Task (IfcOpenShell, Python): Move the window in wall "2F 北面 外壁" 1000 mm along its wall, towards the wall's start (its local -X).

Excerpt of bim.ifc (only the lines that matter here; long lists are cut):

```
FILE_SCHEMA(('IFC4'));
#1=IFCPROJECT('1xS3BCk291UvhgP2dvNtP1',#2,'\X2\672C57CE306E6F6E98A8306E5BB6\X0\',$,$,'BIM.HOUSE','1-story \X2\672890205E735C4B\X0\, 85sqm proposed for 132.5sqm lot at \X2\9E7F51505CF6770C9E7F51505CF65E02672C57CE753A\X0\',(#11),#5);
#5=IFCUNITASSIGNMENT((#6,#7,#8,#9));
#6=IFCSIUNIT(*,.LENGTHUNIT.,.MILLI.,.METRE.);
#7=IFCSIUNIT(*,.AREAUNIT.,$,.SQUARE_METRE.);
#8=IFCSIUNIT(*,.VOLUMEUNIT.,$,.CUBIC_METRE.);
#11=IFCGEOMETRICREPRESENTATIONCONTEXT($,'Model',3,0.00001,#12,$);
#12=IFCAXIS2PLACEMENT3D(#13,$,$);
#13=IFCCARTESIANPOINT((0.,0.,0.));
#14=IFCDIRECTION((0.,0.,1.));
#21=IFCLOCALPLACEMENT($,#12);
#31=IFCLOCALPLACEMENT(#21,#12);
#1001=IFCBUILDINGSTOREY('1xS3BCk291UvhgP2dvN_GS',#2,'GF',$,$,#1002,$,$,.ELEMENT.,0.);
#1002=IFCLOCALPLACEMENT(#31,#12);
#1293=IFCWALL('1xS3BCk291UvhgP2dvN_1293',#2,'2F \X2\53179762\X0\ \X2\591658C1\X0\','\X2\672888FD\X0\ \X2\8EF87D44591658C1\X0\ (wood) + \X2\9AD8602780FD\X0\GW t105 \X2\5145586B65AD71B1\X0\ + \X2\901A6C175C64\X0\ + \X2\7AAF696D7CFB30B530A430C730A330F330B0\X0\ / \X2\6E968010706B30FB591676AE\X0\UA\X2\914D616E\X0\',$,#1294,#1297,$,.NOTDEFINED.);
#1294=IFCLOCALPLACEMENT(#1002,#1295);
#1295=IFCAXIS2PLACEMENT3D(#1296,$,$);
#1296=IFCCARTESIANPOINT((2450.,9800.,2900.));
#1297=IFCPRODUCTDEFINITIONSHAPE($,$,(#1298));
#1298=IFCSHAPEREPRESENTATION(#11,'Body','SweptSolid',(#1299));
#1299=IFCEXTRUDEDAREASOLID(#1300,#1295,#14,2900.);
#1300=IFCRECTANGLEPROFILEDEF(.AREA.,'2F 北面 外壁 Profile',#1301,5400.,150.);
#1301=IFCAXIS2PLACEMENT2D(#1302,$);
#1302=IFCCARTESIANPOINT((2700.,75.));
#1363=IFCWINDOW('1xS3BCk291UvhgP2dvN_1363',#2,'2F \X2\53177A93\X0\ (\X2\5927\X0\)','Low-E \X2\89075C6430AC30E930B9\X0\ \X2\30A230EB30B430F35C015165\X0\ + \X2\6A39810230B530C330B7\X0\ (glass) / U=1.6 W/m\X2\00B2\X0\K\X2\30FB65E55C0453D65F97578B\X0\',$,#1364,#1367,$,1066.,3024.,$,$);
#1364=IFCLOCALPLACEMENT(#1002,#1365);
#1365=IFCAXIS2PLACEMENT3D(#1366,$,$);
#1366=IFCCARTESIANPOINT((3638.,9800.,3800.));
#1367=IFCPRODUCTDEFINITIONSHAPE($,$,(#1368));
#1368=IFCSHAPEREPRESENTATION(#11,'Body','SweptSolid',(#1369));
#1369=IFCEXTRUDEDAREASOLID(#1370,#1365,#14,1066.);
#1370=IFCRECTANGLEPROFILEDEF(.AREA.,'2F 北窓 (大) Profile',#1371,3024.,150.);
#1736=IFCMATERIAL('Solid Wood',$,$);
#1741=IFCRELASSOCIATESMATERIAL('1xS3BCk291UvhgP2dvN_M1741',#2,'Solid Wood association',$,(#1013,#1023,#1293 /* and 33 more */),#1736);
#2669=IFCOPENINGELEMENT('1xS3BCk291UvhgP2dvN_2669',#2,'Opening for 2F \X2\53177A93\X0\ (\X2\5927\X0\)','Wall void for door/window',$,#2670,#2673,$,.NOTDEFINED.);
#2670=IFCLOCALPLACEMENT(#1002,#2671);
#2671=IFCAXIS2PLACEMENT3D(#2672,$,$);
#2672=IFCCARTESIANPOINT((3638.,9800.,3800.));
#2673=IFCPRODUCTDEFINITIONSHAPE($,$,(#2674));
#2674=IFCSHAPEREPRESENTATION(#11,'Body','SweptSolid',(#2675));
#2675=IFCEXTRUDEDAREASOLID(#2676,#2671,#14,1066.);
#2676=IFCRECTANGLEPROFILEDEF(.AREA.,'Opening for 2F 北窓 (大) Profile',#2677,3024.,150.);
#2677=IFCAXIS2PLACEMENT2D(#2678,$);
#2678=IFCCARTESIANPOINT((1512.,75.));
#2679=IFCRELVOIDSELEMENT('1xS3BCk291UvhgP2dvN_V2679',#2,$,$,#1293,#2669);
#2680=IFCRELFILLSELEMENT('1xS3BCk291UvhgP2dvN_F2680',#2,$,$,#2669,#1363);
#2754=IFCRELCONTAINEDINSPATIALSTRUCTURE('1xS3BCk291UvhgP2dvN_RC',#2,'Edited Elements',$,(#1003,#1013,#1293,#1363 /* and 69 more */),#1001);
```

```python
import ifcopenshell
import ifcopenshell.api.geometry
import ifcopenshell.util.placement
import ifcopenshell.util.unit

model = ifcopenshell.open("bim.ifc")
unit_scale = ifcopenshell.util.unit.calculate_unit_scale(model)

window = model.by_id(1363)
opening = window.FillsVoids[0].RelatingOpeningElement
wall = opening.VoidsElements[0].RelatingBuildingElement

wall_matrix = ifcopenshell.util.placement.get_local_placement(wall.ObjectPlacement)
shift = wall_matrix[:3, 0] * -1 / unit_scale
before = ifcopenshell.util.placement.get_local_placement(window.ObjectPlacement)[:3, 3].copy()

# The window is not placed relative to its opening, so move both.
for product in (opening, window):
    matrix = ifcopenshell.util.placement.get_local_placement(product.ObjectPlacement)
    matrix[:3, 3] += shift
    ifcopenshell.api.geometry.edit_object_placement(model, product=product, matrix=matrix, is_si=False)

after = ifcopenshell.util.placement.get_local_placement(window.ObjectPlacement)[:3, 3]
print("window moved by", (after - before).round(3) + 0.0)

model.write("bim_v2.ifc")
```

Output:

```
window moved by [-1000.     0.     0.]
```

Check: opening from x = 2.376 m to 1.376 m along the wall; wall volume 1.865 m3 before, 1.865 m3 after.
